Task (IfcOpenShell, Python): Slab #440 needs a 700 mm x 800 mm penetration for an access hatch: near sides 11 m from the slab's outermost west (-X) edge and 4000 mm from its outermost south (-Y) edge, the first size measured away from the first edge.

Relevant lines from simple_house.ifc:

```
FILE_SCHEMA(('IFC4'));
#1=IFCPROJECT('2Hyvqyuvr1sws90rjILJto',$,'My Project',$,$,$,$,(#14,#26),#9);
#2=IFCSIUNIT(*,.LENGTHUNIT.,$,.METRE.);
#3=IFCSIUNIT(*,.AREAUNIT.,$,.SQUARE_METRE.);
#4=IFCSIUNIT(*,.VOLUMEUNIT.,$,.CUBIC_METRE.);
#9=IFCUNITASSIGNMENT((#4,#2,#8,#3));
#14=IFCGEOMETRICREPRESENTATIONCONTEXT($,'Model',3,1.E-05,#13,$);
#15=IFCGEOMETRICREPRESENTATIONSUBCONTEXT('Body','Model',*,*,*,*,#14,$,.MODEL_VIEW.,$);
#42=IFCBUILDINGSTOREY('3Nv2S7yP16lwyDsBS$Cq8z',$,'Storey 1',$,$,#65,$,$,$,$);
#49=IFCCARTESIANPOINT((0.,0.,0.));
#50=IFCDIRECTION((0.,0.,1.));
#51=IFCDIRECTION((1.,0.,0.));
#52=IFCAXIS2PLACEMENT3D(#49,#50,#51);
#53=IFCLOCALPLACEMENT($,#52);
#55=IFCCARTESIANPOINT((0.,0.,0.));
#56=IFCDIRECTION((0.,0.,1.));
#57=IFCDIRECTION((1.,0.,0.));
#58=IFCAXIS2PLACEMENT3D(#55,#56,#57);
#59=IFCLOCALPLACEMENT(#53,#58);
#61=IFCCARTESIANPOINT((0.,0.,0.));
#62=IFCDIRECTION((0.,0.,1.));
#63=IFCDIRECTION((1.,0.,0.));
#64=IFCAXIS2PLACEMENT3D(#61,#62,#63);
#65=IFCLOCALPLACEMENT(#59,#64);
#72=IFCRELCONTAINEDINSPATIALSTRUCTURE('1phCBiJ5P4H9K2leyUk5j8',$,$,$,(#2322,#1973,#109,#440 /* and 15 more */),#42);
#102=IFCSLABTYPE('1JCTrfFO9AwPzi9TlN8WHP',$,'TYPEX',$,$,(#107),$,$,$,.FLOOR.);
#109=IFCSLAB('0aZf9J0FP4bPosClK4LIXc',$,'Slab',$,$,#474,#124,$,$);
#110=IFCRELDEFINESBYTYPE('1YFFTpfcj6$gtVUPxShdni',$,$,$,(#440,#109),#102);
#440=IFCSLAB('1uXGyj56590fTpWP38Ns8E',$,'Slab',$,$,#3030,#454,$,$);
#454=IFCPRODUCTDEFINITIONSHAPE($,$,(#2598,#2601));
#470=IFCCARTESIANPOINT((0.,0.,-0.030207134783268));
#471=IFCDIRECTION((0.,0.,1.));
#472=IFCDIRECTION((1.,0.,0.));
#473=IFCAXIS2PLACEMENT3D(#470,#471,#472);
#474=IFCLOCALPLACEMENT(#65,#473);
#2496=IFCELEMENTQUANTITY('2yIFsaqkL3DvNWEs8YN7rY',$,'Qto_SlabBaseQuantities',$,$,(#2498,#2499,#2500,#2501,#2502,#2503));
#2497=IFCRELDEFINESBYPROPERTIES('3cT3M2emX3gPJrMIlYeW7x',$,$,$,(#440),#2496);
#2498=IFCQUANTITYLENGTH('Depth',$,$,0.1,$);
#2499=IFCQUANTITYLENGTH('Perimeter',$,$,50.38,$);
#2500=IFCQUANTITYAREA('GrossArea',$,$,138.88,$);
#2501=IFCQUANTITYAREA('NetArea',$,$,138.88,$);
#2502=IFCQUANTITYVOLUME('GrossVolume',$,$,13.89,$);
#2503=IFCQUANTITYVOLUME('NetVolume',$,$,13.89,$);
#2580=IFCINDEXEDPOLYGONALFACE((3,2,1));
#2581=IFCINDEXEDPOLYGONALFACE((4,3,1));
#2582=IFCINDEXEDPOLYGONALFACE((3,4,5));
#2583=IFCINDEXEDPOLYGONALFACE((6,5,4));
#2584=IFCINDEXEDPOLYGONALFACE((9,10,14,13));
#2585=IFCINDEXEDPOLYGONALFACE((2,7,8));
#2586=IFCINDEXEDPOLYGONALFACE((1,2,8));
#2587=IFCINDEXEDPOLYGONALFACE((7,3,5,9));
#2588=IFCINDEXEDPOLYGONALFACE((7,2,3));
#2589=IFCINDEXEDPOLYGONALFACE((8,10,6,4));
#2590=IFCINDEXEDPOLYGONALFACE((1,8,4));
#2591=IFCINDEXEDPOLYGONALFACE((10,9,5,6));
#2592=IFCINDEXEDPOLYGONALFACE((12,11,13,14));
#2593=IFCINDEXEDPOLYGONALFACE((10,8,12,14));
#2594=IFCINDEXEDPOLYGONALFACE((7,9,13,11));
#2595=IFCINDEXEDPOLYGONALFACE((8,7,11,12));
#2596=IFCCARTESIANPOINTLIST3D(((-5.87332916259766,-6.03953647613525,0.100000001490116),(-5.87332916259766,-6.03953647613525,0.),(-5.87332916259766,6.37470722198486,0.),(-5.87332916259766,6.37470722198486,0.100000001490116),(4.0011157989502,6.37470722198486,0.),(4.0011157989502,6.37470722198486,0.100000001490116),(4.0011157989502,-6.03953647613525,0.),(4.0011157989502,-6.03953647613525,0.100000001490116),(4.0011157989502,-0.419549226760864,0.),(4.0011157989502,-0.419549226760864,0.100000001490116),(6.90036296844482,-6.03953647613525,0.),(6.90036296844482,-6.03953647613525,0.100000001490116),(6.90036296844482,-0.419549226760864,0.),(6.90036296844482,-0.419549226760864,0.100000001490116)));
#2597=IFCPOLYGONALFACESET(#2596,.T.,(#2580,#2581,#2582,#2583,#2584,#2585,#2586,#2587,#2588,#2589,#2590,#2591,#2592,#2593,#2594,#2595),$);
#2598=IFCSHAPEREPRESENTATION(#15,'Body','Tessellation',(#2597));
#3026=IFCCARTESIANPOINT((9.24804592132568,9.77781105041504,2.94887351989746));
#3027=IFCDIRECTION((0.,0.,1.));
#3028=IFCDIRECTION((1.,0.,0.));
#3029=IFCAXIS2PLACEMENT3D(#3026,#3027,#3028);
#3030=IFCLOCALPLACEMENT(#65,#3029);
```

```python
import numpy as np
import ifcopenshell
import ifcopenshell.api.feature
import ifcopenshell.api.geometry
import ifcopenshell.api.pset
import ifcopenshell.api.root
import ifcopenshell.geom
import ifcopenshell.util.element
import ifcopenshell.util.placement
import ifcopenshell.util.representation
import ifcopenshell.util.shape
import ifcopenshell.util.unit

model = ifcopenshell.open("simple_house.ifc")
unit_scale = ifcopenshell.util.unit.calculate_unit_scale(model)
area_scale = ifcopenshell.util.unit.calculate_unit_scale(model, "AREAUNIT")
volume_scale = ifcopenshell.util.unit.calculate_unit_scale(model, "VOLUMEUNIT")
settings = ifcopenshell.geom.settings()


def volume(element):
    """Net volume in cubic metres, openings subtracted."""
    shape = ifcopenshell.geom.create_shape(settings, element)
    return ifcopenshell.util.shape.get_volume(shape.geometry)


slab = model.by_guid("1uXGyj56590fTpWP38Ns8E")
before = volume(slab)

# Extent in the slab's own axes, in metres. The edges named are its -X and -Y sides.
slab_shape = ifcopenshell.geom.create_shape(settings, slab)
vertices = ifcopenshell.util.shape.get_vertices(slab_shape.geometry)
x_min, y_min, bottom = vertices.min(axis=0)
top = vertices[:, 2].max()

opening = ifcopenshell.api.root.create_entity(model, ifc_class="IfcOpeningElement", name="Access hatch opening", predefined_type="OPENING")
context = ifcopenshell.util.representation.get_context(model, "Model", "Body", "MODEL_VIEW")
width, depth = 0.7, 0.8
outline = [(0.0, 0.0), (width, 0.0), (width, depth), (0.0, depth), (0.0, 0.0)]
# Overshoot both faces by 50 mm so the cut is clean.
shape = ifcopenshell.api.geometry.add_slab_representation(
    model, context=context, depth=top - bottom + 0.1, polyline=outline
)
ifcopenshell.api.geometry.assign_representation(model, product=opening, representation=shape)

matrix = ifcopenshell.util.placement.get_local_placement(slab.ObjectPlacement)
matrix[:, 3] = matrix @ np.append(np.array([x_min + 11, y_min + 4, bottom - 0.05]) / unit_scale, 1.0)
ifcopenshell.api.geometry.edit_object_placement(model, product=opening, matrix=matrix, is_si=False)
ifcopenshell.api.feature.add_feature(model, feature=opening, element=slab)

after = volume(slab)

# Update the slab's stored quantities.
qto = model.by_id(ifcopenshell.util.element.get_pset(slab, "Qto_SlabBaseQuantities", should_inherit=False)["id"])
ifcopenshell.api.pset.edit_qto(model, qto=qto, properties={
    "NetArea": after / (top - bottom) / area_scale,
    "NetVolume": after / volume_scale,
})

print(f"slab volume {before:.3f} -> {after:.3f} m3")

model.write("simple_house_v2.ifc")
```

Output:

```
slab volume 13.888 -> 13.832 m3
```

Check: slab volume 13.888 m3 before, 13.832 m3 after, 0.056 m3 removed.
